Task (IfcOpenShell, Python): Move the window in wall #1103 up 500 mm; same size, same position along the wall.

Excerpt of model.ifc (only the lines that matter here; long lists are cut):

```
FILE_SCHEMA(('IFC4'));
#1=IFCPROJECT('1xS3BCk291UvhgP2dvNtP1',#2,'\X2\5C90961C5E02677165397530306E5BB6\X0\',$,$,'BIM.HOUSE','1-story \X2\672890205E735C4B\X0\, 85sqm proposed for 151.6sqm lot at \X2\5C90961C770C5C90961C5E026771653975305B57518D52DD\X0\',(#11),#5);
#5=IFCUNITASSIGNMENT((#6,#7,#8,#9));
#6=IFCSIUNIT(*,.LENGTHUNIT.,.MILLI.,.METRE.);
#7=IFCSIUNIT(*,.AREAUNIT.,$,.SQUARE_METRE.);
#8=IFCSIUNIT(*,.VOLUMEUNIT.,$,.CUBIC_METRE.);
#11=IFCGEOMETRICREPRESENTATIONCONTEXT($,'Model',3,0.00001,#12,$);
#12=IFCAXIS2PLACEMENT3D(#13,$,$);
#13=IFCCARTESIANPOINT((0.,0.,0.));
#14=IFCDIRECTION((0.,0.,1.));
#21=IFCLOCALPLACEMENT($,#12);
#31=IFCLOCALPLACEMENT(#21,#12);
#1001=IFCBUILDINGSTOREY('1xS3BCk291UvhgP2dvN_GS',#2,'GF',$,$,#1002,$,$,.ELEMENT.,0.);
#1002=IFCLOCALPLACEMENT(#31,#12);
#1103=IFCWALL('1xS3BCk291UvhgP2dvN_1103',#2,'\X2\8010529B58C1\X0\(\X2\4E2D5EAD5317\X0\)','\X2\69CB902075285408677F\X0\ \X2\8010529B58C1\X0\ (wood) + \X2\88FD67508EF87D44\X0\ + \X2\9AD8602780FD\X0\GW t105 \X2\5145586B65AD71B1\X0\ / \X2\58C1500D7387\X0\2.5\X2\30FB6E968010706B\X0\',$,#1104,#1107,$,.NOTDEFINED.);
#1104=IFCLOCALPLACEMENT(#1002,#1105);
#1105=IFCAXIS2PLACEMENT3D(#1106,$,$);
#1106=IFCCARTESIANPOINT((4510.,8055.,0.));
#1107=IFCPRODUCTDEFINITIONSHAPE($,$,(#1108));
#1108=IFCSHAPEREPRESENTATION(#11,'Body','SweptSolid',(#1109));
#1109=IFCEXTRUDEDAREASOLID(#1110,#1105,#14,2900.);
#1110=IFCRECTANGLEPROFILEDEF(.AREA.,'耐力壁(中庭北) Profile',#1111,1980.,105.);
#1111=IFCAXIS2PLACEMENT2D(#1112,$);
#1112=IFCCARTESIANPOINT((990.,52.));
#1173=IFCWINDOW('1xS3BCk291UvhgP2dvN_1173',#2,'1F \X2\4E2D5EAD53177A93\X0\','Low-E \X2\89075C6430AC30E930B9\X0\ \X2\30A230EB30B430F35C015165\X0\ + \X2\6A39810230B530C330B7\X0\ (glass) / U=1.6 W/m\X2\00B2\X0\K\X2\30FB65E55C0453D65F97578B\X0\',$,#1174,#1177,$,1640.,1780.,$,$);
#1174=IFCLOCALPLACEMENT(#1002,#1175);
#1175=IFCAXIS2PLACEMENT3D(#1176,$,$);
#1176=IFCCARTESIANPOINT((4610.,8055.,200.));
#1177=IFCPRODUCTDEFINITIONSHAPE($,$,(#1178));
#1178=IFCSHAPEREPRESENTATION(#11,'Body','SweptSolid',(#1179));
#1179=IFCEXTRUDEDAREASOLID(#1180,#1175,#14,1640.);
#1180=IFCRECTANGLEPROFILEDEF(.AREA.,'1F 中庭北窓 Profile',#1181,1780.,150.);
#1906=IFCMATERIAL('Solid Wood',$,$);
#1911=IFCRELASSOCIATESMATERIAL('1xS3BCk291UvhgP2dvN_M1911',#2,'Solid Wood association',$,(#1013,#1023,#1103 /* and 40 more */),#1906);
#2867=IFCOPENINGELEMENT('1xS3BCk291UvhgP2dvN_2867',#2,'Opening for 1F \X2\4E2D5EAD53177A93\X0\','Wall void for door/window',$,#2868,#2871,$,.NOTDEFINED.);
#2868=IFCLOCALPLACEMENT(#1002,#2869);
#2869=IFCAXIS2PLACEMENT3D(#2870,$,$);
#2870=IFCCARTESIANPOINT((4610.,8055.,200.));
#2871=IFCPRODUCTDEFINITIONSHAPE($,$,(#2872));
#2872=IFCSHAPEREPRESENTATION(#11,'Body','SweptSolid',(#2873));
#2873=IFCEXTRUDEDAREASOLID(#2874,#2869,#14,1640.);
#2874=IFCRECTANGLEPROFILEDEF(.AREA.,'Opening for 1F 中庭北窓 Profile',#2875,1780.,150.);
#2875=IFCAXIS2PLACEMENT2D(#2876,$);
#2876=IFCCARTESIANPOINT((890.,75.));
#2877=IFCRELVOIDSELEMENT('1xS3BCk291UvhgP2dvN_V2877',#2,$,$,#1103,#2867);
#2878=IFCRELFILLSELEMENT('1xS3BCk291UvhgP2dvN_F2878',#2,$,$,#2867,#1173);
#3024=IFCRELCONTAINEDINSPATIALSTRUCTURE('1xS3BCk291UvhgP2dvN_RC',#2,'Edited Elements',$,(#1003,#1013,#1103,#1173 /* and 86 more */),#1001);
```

```python
import numpy as np
import ifcopenshell
import ifcopenshell.api.geometry
import ifcopenshell.util.placement
import ifcopenshell.util.unit

model = ifcopenshell.open("model.ifc")
unit_scale = ifcopenshell.util.unit.calculate_unit_scale(model)

window = model.by_guid("1xS3BCk291UvhgP2dvN_1173")
opening = window.FillsVoids[0].RelatingOpeningElement
dz = 0.5 / unit_scale

shift = np.array([0.0, 0.0, dz])
# The window is not placed relative to its opening, so move both.
for product in (opening, window):
    matrix = ifcopenshell.util.placement.get_local_placement(product.ObjectPlacement)
    matrix[:3, 3] += shift
    ifcopenshell.api.geometry.edit_object_placement(model, product=product, matrix=matrix, is_si=False)

print(f"moved by {dz * unit_scale:+.3f} m")

model.write("model_updated.ifc")
```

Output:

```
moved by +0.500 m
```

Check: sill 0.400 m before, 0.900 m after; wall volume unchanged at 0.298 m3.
